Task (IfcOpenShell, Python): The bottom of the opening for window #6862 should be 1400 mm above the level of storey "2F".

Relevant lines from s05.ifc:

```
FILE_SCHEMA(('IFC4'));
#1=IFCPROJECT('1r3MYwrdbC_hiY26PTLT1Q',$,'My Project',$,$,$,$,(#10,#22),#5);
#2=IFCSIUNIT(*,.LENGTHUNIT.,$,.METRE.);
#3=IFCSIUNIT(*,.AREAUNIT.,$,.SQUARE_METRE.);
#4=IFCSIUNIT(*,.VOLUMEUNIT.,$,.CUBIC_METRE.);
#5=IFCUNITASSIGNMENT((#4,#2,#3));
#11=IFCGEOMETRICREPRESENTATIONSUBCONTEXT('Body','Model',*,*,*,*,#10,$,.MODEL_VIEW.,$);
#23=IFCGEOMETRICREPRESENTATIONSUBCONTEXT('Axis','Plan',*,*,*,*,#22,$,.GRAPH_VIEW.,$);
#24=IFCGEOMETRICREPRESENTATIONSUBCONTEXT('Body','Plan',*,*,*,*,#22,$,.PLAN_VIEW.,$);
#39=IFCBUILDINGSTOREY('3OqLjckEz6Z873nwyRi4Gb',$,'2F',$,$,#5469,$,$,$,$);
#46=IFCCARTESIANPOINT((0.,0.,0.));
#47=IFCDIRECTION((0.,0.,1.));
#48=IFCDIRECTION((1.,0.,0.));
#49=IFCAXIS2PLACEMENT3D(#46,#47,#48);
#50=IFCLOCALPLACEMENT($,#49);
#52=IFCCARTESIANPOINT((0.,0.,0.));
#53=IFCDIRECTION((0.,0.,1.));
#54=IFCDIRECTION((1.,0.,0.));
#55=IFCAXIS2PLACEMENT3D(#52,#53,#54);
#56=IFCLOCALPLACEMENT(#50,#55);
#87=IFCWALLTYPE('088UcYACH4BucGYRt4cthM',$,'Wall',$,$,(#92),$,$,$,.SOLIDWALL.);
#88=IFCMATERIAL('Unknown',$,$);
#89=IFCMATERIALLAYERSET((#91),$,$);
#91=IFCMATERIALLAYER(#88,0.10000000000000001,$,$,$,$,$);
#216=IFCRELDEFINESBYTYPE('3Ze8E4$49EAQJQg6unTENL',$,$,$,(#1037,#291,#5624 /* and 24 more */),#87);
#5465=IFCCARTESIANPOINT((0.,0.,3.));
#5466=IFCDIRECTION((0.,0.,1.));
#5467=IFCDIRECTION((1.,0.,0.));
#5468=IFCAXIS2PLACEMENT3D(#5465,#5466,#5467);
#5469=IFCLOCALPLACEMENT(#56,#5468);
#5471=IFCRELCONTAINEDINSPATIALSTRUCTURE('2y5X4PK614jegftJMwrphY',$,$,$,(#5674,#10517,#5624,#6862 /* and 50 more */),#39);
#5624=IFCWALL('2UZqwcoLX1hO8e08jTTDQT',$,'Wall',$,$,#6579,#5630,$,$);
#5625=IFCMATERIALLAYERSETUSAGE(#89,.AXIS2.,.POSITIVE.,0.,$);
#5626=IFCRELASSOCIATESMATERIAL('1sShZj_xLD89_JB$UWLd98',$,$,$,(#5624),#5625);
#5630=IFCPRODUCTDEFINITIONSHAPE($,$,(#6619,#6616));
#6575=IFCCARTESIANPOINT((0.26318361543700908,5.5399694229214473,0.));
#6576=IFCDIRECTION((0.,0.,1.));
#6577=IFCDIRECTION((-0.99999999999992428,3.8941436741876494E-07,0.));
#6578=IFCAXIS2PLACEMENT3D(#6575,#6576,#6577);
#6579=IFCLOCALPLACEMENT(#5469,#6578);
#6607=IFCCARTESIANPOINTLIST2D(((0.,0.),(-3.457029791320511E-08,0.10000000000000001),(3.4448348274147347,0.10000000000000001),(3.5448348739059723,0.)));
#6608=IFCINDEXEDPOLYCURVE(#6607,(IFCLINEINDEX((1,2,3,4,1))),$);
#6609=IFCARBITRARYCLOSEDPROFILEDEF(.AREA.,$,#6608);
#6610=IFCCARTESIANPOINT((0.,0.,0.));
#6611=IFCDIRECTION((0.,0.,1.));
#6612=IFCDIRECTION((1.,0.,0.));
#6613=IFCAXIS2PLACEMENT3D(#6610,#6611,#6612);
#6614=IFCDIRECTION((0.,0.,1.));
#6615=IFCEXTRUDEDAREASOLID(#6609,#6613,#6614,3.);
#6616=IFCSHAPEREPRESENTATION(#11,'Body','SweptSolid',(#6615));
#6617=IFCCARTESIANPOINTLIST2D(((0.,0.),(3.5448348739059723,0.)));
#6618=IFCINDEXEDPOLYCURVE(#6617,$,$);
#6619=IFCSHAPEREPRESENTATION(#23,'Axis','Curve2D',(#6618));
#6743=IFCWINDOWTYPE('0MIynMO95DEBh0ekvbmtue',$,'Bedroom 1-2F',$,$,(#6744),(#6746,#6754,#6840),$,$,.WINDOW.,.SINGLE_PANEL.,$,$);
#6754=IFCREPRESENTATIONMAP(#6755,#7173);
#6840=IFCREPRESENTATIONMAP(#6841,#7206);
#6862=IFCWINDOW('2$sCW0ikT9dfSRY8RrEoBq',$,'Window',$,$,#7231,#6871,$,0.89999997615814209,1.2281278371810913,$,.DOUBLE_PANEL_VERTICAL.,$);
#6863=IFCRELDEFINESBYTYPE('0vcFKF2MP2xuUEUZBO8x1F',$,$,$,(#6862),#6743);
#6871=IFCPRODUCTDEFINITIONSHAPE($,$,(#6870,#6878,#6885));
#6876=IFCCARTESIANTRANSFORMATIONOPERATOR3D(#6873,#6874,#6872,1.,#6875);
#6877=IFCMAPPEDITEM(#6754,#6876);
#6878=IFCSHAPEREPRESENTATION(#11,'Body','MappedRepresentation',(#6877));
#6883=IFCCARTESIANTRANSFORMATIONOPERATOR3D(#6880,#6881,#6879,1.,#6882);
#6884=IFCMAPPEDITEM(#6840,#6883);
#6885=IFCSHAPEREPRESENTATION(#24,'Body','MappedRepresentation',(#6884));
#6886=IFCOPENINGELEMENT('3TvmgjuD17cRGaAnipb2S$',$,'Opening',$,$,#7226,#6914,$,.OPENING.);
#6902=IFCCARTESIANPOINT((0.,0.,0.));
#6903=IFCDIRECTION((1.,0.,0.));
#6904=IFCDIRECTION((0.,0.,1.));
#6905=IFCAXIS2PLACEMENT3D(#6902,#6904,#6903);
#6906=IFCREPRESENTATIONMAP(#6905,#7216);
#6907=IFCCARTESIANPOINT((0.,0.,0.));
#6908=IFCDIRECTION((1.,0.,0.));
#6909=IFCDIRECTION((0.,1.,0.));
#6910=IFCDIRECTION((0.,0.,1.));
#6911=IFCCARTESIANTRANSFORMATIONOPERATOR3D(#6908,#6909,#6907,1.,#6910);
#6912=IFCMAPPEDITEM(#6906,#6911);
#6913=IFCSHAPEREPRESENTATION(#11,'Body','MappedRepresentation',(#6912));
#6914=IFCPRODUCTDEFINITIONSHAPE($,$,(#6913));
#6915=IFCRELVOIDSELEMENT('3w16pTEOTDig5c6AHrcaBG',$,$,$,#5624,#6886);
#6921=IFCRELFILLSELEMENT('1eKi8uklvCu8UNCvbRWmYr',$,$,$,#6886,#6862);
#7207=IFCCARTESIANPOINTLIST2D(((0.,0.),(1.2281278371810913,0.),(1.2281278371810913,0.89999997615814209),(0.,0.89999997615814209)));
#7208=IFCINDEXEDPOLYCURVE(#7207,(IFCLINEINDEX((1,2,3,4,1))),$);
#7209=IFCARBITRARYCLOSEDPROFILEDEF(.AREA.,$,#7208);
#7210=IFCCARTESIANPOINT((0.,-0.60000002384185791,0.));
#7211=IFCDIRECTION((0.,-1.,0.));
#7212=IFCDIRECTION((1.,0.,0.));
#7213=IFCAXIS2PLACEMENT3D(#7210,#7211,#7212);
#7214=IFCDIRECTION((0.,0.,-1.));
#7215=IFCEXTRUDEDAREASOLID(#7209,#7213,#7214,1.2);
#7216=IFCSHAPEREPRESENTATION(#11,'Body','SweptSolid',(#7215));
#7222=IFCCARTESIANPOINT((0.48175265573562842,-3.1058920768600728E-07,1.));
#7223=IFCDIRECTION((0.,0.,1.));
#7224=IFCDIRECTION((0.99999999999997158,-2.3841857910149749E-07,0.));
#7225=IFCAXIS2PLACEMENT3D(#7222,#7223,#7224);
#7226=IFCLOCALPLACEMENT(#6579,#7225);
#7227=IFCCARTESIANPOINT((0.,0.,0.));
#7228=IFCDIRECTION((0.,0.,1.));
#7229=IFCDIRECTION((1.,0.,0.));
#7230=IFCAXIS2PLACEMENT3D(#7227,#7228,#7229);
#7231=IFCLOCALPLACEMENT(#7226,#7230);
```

```python
import numpy as np
import ifcopenshell
import ifcopenshell.api.geometry
import ifcopenshell.geom
import ifcopenshell.util.element
import ifcopenshell.util.placement
import ifcopenshell.util.shape
import ifcopenshell.util.unit

model = ifcopenshell.open("s05.ifc")
unit_scale = ifcopenshell.util.unit.calculate_unit_scale(model)

window = model.by_guid("2$sCW0ikT9dfSRY8RrEoBq")
opening = window.FillsVoids[0].RelatingOpeningElement
storey = ifcopenshell.util.element.get_container(window, ifc_class="IfcBuildingStorey")
level = ifcopenshell.util.placement.get_local_placement(storey.ObjectPlacement)[2, 3]

# The opening's origin need not be at the sill, so measure its lowest point.
shape = ifcopenshell.geom.create_shape(ifcopenshell.geom.settings(), opening)
bottom = ifcopenshell.util.shape.get_shape_bottom_elevation(shape, shape.geometry) / unit_scale
dz = level + 1.4 / unit_scale - bottom

shift = np.array([0.0, 0.0, dz])
# The window is placed relative to its opening, so it follows when the opening moves.
matrix = ifcopenshell.util.placement.get_local_placement(opening.ObjectPlacement)
matrix[:3, 3] += shift
ifcopenshell.api.geometry.edit_object_placement(
    model, product=opening, matrix=matrix, is_si=False, should_transform_children=True
)

print(f"moved by {dz * unit_scale:+.3f} m")

model.write("s05_edited.ifc")
```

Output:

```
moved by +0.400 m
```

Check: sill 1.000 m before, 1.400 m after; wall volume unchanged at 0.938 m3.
